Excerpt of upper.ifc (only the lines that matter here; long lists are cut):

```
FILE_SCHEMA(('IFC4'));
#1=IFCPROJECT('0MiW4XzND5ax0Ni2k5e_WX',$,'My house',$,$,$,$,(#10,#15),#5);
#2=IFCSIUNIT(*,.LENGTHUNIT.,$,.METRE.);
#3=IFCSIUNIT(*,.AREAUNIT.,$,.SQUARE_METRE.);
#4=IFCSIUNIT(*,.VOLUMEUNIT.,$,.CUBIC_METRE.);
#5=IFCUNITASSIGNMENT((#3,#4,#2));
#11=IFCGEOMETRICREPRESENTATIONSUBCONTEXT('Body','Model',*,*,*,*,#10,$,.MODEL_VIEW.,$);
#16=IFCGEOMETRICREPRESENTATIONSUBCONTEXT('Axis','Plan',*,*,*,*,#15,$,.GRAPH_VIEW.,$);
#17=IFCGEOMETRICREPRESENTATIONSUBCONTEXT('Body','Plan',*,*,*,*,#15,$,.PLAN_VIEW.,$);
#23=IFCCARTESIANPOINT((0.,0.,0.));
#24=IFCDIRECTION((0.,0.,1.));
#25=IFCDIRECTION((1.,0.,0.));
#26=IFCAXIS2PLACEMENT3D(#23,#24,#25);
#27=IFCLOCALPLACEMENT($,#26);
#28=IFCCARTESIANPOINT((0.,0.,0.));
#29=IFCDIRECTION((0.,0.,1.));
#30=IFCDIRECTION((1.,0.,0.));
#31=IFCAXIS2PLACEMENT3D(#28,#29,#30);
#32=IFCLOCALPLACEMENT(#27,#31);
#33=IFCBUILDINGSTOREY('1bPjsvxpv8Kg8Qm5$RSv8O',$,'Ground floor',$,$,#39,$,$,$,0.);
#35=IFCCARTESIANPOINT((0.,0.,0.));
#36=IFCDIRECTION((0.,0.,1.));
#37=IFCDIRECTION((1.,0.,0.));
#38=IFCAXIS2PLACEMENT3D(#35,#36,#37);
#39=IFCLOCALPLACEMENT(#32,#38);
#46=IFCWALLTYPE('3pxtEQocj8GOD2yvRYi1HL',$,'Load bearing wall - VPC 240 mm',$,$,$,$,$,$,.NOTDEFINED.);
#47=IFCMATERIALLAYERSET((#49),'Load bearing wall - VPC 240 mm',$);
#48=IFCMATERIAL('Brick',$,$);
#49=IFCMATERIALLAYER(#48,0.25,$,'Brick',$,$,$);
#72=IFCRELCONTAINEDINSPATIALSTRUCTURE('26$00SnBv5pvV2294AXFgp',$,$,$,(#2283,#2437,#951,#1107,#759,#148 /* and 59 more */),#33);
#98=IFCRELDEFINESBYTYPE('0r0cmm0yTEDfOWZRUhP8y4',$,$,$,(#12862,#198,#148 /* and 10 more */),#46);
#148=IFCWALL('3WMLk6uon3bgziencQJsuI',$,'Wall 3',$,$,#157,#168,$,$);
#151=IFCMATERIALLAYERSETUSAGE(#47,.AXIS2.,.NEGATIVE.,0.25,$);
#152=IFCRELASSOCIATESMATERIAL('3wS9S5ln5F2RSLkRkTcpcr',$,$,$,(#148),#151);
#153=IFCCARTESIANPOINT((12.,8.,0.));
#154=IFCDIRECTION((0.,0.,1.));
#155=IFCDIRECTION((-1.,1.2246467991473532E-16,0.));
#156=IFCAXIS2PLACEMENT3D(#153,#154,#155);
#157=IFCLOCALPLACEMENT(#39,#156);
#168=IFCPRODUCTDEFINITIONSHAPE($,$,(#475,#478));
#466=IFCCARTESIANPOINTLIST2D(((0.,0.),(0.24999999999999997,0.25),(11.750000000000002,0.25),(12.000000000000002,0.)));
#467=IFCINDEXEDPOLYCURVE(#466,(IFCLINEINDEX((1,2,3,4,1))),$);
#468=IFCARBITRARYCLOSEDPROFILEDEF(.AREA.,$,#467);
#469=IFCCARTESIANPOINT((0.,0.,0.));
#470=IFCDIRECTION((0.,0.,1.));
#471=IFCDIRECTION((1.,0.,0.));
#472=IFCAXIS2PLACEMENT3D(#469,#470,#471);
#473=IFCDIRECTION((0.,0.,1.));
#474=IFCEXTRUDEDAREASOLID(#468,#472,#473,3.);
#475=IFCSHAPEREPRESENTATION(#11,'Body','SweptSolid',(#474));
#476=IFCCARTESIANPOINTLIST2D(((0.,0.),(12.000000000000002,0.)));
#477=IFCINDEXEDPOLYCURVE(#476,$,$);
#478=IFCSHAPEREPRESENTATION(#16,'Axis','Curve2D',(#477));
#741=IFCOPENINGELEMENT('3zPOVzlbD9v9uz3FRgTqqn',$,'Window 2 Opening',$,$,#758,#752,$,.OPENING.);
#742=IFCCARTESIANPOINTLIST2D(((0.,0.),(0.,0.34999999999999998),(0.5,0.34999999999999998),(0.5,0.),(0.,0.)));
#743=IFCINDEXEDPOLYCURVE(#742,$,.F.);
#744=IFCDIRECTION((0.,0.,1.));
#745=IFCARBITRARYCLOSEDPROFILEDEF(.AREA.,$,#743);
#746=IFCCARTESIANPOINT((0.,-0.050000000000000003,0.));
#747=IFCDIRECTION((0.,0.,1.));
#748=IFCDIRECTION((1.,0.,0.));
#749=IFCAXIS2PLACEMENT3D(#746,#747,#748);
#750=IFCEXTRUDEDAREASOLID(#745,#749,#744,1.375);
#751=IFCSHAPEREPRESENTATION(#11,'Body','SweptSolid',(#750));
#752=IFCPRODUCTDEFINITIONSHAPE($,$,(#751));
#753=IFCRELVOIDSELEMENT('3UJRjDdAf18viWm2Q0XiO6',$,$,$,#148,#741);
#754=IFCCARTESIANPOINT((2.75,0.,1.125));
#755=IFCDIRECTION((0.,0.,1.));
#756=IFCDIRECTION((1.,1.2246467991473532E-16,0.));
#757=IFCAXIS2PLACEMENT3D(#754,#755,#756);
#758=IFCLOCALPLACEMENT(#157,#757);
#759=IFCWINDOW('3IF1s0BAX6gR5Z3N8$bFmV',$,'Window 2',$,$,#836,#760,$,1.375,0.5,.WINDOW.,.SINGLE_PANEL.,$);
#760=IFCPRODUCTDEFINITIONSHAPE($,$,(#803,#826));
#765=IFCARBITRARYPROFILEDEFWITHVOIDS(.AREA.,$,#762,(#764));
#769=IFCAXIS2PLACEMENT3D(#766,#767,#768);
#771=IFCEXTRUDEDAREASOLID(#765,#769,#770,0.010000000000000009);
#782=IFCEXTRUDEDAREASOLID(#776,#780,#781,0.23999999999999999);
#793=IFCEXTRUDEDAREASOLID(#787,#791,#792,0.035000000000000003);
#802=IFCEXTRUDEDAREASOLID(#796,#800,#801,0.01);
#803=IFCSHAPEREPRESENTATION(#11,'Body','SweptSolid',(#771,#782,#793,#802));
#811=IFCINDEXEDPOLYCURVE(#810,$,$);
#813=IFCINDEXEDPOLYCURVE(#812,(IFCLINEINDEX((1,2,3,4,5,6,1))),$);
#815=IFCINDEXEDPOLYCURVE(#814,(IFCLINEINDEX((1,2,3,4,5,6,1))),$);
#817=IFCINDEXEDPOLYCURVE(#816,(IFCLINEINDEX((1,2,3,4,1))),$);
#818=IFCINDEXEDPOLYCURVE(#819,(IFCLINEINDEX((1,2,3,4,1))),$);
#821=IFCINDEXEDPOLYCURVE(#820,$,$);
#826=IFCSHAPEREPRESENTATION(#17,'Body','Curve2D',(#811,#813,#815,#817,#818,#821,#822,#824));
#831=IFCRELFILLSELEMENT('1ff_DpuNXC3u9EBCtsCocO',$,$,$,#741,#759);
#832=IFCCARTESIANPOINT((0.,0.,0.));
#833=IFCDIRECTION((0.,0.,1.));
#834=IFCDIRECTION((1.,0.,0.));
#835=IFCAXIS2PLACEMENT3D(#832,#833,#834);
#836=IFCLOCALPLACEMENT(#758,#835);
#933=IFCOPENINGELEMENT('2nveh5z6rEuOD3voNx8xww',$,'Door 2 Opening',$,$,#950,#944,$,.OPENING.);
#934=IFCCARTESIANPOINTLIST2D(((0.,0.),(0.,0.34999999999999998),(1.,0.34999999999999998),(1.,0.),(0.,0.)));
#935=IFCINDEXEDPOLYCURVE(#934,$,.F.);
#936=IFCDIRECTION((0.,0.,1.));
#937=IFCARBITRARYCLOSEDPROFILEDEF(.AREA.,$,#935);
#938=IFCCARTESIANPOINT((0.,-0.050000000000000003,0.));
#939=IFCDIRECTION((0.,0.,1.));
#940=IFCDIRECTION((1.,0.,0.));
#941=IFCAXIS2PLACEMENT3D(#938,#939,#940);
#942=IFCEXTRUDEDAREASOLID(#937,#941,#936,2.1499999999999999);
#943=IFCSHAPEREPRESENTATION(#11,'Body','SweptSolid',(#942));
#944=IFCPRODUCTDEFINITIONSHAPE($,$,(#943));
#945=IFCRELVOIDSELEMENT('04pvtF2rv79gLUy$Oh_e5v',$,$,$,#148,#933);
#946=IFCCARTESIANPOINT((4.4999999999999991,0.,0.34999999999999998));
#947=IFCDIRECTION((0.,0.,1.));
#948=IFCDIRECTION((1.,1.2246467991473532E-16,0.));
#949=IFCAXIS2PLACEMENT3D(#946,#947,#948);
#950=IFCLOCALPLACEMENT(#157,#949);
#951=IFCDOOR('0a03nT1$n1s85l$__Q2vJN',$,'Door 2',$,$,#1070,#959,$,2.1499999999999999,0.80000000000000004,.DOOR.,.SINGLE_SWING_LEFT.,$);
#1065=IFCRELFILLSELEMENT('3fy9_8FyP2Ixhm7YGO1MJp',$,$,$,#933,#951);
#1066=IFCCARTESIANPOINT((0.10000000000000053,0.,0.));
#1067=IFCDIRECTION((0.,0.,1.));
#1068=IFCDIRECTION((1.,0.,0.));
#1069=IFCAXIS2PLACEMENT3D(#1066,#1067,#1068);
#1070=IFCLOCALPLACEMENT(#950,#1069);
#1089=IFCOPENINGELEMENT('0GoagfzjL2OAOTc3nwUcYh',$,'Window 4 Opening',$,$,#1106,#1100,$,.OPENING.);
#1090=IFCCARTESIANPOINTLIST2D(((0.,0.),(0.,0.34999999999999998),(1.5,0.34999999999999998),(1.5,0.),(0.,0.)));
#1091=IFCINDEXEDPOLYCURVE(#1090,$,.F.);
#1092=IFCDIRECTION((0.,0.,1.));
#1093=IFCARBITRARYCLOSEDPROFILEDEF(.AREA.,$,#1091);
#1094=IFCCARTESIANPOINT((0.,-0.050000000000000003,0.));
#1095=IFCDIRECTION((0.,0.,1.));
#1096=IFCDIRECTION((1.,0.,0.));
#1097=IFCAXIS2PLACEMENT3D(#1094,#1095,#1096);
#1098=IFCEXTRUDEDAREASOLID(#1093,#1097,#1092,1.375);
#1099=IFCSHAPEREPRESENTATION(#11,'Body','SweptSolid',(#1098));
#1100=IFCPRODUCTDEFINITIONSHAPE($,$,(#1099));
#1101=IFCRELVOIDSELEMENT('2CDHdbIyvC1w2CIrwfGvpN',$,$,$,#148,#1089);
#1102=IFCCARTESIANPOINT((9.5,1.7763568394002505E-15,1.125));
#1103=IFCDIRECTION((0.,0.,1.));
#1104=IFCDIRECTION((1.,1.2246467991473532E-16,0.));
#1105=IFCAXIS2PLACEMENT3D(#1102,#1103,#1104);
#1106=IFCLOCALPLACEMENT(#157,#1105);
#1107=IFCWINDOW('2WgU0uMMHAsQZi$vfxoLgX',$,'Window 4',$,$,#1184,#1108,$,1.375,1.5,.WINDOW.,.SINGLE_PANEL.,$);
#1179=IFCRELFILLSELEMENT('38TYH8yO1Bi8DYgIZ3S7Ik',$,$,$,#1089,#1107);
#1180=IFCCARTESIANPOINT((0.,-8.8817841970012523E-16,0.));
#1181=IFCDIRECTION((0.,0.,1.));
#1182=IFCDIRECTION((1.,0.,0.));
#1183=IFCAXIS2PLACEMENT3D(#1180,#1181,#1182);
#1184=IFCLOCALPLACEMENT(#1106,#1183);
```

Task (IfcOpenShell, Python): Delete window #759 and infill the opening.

```python
import ifcopenshell
import ifcopenshell.api.feature
import ifcopenshell.api.root
import ifcopenshell.geom
import ifcopenshell.util.shape

model = ifcopenshell.open("upper.ifc")
settings = ifcopenshell.geom.settings()


def volume(element):
    """Net volume in cubic metres, openings subtracted."""
    shape = ifcopenshell.geom.create_shape(settings, element)
    return ifcopenshell.util.shape.get_volume(shape.geometry)


window = model.by_guid("3IF1s0BAX6gR5Z3N8$bFmV")
opening = window.FillsVoids[0].RelatingOpeningElement
wall = opening.VoidsElements[0].RelatingBuildingElement
before = volume(wall)

ifcopenshell.api.root.remove_product(model, product=window)
ifcopenshell.api.feature.remove_feature(model, feature=opening)

after = volume(wall)

print(f"wall volume {before:.3f} -> {after:.3f} m3")

model.write("upper_rev.ifc")
```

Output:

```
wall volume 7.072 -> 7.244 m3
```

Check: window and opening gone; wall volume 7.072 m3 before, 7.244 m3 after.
